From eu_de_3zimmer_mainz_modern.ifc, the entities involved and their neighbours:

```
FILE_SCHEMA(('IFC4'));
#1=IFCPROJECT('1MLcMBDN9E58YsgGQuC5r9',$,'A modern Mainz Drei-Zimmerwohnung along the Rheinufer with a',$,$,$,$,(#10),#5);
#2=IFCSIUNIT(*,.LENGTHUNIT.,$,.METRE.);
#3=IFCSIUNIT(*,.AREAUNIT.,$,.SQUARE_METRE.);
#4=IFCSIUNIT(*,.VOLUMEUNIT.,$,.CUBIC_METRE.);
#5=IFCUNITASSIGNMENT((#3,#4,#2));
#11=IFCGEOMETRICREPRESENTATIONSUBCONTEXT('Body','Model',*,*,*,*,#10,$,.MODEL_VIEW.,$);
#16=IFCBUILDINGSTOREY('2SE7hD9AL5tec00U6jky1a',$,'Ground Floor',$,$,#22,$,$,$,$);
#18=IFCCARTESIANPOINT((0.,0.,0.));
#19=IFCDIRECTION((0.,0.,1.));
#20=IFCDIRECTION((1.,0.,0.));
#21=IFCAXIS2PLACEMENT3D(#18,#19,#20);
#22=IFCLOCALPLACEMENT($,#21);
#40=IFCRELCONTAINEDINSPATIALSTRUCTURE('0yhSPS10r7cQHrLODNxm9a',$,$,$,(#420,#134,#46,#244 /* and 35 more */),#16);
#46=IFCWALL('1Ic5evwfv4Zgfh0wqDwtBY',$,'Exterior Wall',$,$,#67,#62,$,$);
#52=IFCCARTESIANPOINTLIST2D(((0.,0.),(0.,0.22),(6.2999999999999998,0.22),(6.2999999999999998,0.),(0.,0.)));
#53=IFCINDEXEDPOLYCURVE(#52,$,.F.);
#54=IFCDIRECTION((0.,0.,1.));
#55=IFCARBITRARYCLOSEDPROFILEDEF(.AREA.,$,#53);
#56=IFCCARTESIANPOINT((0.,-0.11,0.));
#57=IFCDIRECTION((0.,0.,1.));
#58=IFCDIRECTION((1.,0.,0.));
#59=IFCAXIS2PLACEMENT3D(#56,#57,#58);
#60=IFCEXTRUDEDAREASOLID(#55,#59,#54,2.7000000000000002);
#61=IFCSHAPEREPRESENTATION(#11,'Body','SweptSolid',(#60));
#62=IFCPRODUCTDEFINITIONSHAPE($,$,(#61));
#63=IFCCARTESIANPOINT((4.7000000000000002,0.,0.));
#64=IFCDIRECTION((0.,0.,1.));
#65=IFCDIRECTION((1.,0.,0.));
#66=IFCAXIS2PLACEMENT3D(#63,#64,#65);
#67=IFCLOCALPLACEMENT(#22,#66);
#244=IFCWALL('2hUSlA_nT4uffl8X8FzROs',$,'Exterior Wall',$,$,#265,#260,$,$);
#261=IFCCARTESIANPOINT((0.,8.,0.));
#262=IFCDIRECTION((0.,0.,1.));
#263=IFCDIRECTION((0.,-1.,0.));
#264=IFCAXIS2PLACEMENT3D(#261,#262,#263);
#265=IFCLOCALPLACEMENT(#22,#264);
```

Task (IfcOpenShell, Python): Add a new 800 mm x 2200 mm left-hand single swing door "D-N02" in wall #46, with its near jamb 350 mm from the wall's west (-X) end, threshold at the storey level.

```python
import numpy as np
import ifcopenshell
import ifcopenshell.api.feature
import ifcopenshell.api.geometry
import ifcopenshell.api.root
import ifcopenshell.api.spatial
import ifcopenshell.geom
import ifcopenshell.util.element
import ifcopenshell.util.placement
import ifcopenshell.util.representation
import ifcopenshell.util.shape
import ifcopenshell.util.unit

model = ifcopenshell.open("eu_de_3zimmer_mainz_modern.ifc")
unit_scale = ifcopenshell.util.unit.calculate_unit_scale(model)
settings = ifcopenshell.geom.settings()


def volume(element):
    """Net volume in cubic metres, openings subtracted."""
    shape = ifcopenshell.geom.create_shape(settings, element)
    return ifcopenshell.util.shape.get_volume(shape.geometry)


wall = model.by_guid("1Ic5evwfv4Zgfh0wqDwtBY")
storey = ifcopenshell.util.element.get_container(wall, ifc_class="IfcBuildingStorey")
context = ifcopenshell.util.representation.get_context(model, "Model", "Body", "MODEL_VIEW")
before = volume(wall)

width, height, from_end, sill = 0.8, 2.2, 0.35, 0.0  # metres

# The wall runs along its own X axis, and the end named is its -X end.
wall_shape = ifcopenshell.geom.create_shape(settings, wall)
x, y, z = ifcopenshell.util.shape.get_vertices(wall_shape.geometry).T
start = x.min() + from_end
face, thickness = float(y.min()), float(y.max() - y.min())
wall_matrix = ifcopenshell.util.placement.get_local_placement(wall.ObjectPlacement)
level = ifcopenshell.util.placement.get_local_placement(storey.ObjectPlacement)[2, 3]


def in_wall(x, y):
    """Placement at x, y metres in the wall's axes, at sill height."""
    matrix = wall_matrix.copy()
    matrix[:, 3] = wall_matrix @ np.array([x / unit_scale, y / unit_scale, 0.0, 1.0])
    matrix[2, 3] = level + sill / unit_scale
    return matrix


# Opening: a box that overshoots both wall faces by 50 mm.
opening = ifcopenshell.api.root.create_entity(model, ifc_class="IfcOpeningElement", predefined_type="OPENING")
box = ifcopenshell.api.geometry.add_wall_representation(
    model, context=context, length=width, height=height, thickness=thickness + 0.1
)
ifcopenshell.api.geometry.assign_representation(model, product=opening, representation=box)
ifcopenshell.api.geometry.edit_object_placement(model, product=opening, matrix=in_wall(start, face - 0.05), is_si=False)
ifcopenshell.api.feature.add_feature(model, feature=opening, element=wall)

door = ifcopenshell.api.root.create_entity(model, ifc_class="IfcDoor", name="D-N02", predefined_type="DOOR")
door.OverallWidth, door.OverallHeight = width / unit_scale, height / unit_scale
door.OperationType = "SINGLE_SWING_LEFT"
body = ifcopenshell.api.geometry.add_door_representation(
    model,
    context=context,
    overall_width=door.OverallWidth,
    overall_height=door.OverallHeight,
    operation_type="SINGLE_SWING_LEFT",
    lining_properties={"LiningDepth": thickness / unit_scale, "ThresholdDepth": thickness / unit_scale},
)
ifcopenshell.api.geometry.assign_representation(model, product=door, representation=body)
ifcopenshell.api.spatial.assign_container(model, products=[door], relating_structure=storey)
ifcopenshell.api.feature.add_filling(model, opening=opening, element=door)

# The lining spans the wall, so the door starts at the wall face.
ifcopenshell.api.geometry.edit_object_placement(model, product=door, matrix=in_wall(start, face), is_si=False)

after = volume(wall)

print(f"wall volume {before:.3f} -> {after:.3f} m3")

model.write("eu_de_3zimmer_mainz_modern-out.ifc")
```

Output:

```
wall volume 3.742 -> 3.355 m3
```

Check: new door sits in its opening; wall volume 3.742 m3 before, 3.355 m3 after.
